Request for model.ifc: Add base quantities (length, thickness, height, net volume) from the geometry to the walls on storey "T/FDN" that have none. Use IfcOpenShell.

First a look at what the model holds.

```python
import ifcopenshell
import ifcopenshell.util.element
import ifcopenshell.util.unit

model = ifcopenshell.open("model.ifc")
print(model.schema)
for unit_type in ("LENGTHUNIT", "AREAUNIT", "VOLUMEUNIT"):
    print(unit_type, ifcopenshell.util.unit.calculate_unit_scale(model, unit_type))
storey = next(s for s in model.by_type("IfcBuildingStorey") if s.Name == "T/FDN")
walls = [e for e in ifcopenshell.util.element.get_decomposition(storey) if e.is_a("IfcWall")]
for e in sorted(walls, key=lambda e: e.id()):
    print(e.id(), e.is_a(), e.Name, list(ifcopenshell.util.element.get_psets(e, qtos_only=True)), sep=" | ")
```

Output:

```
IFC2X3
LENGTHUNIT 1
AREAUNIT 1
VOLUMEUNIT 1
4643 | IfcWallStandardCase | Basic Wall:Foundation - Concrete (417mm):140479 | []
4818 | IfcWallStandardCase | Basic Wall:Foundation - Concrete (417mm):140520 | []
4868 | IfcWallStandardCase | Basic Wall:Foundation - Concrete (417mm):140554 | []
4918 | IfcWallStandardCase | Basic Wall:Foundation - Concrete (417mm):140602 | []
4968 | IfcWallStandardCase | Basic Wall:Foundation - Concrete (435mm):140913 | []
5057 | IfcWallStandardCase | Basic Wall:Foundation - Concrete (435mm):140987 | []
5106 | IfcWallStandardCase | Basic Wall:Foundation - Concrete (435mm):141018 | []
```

```python
import ifcopenshell
import ifcopenshell.api.pset
import ifcopenshell.geom
import ifcopenshell.util.element
import ifcopenshell.util.shape
import ifcopenshell.util.unit

model = ifcopenshell.open("model.ifc")
unit_scale = ifcopenshell.util.unit.calculate_unit_scale(model)
volume_scale = ifcopenshell.util.unit.calculate_unit_scale(model, "VOLUMEUNIT")
settings = ifcopenshell.geom.settings()

storey = next(s for s in model.by_type("IfcBuildingStorey") if s.Name == "T/FDN")
walls = [e for e in ifcopenshell.util.element.get_decomposition(storey) if e.is_a("IfcWall")]

for e in sorted(walls, key=lambda e: e.id()):
    if ifcopenshell.util.element.get_psets(e, qtos_only=True, should_inherit=False):
        continue
    # Geometry comes back in metres, in the element's own axes.
    shape = ifcopenshell.geom.create_shape(settings, e)
    values = {
        "Length": ifcopenshell.util.shape.get_x(shape.geometry) / unit_scale,
        "Width": ifcopenshell.util.shape.get_y(shape.geometry) / unit_scale,
        "Height": ifcopenshell.util.shape.get_z(shape.geometry) / unit_scale,
        "NetVolume": ifcopenshell.util.shape.get_volume(shape.geometry) / volume_scale,
    }
    qto = ifcopenshell.api.pset.add_qto(model, product=e, name="BaseQuantities")
    ifcopenshell.api.pset.edit_qto(model, qto=qto, properties=values)
    print(e.id(), {k: round(v, 3) for k, v in values.items()})

model.write("model_updated.ifc")
```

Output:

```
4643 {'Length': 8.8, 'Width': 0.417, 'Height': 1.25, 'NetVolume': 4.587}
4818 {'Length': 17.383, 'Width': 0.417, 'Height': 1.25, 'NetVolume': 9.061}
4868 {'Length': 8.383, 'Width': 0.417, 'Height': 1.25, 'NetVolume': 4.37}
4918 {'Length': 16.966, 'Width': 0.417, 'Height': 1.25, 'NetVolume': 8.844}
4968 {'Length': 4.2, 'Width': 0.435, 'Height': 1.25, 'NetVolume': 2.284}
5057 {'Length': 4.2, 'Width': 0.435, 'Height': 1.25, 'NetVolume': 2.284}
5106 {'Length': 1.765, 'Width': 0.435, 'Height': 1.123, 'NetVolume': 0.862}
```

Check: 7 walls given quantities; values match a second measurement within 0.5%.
